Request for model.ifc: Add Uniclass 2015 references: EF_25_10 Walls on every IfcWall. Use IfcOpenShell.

First a look at what the model holds.

```python
import ifcopenshell

model = ifcopenshell.open("model.ifc")
print(model.schema)
print("classifications:", [c.Name for c in model.by_type("IfcClassification")])
for ifc_class in ("IfcDoor", "IfcRoof", "IfcStair", "IfcWall", "IfcWindow"):
    print(ifc_class, len(model.by_type(ifc_class)))
```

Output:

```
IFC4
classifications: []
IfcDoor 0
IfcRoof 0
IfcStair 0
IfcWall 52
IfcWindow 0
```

```python
import ifcopenshell
import ifcopenshell.api.classification

model = ifcopenshell.open("model.ifc")

system = ifcopenshell.api.classification.add_classification(model, classification="Uniclass 2015")

codes = {
    "IfcWall": ("EF_25_10", "Walls"),
}
for ifc_class, (code, name) in codes.items():
    products = model.by_type(ifc_class)
    ifcopenshell.api.classification.add_reference(
        model, products=products, classification=system, identification=code, name=name
    )
    print(code, len(products))

model.write("model_edited.ifc")
```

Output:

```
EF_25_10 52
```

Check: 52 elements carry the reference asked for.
